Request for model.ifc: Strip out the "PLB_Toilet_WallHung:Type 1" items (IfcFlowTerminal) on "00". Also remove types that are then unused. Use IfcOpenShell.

First a look at what the model holds.

```python
import ifcopenshell
import ifcopenshell.util.element

model = ifcopenshell.open("model.ifc")
print(model.schema)
storey = next(s for s in model.by_type("IfcBuildingStorey") if s.Name == "00")
terminals = [e for e in ifcopenshell.util.element.get_decomposition(storey) if e.is_a("IfcFlowTerminal")]
seen = {}
for e in terminals:
    element_type = ifcopenshell.util.element.get_type(e)
    name = element_type.Name if element_type not in (None, e) else None
    seen[name] = seen.get(name, 0) + 1
for name, count in sorted(seen.items(), key=str):
    print(count, "x", name)
```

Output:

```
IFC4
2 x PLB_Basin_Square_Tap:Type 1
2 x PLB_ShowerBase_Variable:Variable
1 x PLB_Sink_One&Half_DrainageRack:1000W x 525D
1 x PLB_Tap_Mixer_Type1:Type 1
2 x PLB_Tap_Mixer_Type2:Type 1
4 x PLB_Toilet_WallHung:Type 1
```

```python
import ifcopenshell
import ifcopenshell.api.root
import ifcopenshell.util.element

model = ifcopenshell.open("model.ifc")

storey = next(s for s in model.by_type("IfcBuildingStorey") if s.Name == "00")
terminals = [e for e in ifcopenshell.util.element.get_decomposition(storey) if e.is_a("IfcFlowTerminal")]
targets = [e for e in terminals if (t := ifcopenshell.util.element.get_type(e)) not in (None, e) and t.Name == "PLB_Toilet_WallHung:Type 1"]
types = {ifcopenshell.util.element.get_type(e) for e in targets} - {None, *targets}

for e in targets:
    ifcopenshell.api.root.remove_product(model, product=e)
print(len(targets), "removed")

unused = [t for t in types if not ifcopenshell.util.element.get_types(t)]
for t in unused:
    ifcopenshell.api.root.remove_product(model, product=t)
print(len(unused), "unused types removed")

model.write("model_rev.ifc")
```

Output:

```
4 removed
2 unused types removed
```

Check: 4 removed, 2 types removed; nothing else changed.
